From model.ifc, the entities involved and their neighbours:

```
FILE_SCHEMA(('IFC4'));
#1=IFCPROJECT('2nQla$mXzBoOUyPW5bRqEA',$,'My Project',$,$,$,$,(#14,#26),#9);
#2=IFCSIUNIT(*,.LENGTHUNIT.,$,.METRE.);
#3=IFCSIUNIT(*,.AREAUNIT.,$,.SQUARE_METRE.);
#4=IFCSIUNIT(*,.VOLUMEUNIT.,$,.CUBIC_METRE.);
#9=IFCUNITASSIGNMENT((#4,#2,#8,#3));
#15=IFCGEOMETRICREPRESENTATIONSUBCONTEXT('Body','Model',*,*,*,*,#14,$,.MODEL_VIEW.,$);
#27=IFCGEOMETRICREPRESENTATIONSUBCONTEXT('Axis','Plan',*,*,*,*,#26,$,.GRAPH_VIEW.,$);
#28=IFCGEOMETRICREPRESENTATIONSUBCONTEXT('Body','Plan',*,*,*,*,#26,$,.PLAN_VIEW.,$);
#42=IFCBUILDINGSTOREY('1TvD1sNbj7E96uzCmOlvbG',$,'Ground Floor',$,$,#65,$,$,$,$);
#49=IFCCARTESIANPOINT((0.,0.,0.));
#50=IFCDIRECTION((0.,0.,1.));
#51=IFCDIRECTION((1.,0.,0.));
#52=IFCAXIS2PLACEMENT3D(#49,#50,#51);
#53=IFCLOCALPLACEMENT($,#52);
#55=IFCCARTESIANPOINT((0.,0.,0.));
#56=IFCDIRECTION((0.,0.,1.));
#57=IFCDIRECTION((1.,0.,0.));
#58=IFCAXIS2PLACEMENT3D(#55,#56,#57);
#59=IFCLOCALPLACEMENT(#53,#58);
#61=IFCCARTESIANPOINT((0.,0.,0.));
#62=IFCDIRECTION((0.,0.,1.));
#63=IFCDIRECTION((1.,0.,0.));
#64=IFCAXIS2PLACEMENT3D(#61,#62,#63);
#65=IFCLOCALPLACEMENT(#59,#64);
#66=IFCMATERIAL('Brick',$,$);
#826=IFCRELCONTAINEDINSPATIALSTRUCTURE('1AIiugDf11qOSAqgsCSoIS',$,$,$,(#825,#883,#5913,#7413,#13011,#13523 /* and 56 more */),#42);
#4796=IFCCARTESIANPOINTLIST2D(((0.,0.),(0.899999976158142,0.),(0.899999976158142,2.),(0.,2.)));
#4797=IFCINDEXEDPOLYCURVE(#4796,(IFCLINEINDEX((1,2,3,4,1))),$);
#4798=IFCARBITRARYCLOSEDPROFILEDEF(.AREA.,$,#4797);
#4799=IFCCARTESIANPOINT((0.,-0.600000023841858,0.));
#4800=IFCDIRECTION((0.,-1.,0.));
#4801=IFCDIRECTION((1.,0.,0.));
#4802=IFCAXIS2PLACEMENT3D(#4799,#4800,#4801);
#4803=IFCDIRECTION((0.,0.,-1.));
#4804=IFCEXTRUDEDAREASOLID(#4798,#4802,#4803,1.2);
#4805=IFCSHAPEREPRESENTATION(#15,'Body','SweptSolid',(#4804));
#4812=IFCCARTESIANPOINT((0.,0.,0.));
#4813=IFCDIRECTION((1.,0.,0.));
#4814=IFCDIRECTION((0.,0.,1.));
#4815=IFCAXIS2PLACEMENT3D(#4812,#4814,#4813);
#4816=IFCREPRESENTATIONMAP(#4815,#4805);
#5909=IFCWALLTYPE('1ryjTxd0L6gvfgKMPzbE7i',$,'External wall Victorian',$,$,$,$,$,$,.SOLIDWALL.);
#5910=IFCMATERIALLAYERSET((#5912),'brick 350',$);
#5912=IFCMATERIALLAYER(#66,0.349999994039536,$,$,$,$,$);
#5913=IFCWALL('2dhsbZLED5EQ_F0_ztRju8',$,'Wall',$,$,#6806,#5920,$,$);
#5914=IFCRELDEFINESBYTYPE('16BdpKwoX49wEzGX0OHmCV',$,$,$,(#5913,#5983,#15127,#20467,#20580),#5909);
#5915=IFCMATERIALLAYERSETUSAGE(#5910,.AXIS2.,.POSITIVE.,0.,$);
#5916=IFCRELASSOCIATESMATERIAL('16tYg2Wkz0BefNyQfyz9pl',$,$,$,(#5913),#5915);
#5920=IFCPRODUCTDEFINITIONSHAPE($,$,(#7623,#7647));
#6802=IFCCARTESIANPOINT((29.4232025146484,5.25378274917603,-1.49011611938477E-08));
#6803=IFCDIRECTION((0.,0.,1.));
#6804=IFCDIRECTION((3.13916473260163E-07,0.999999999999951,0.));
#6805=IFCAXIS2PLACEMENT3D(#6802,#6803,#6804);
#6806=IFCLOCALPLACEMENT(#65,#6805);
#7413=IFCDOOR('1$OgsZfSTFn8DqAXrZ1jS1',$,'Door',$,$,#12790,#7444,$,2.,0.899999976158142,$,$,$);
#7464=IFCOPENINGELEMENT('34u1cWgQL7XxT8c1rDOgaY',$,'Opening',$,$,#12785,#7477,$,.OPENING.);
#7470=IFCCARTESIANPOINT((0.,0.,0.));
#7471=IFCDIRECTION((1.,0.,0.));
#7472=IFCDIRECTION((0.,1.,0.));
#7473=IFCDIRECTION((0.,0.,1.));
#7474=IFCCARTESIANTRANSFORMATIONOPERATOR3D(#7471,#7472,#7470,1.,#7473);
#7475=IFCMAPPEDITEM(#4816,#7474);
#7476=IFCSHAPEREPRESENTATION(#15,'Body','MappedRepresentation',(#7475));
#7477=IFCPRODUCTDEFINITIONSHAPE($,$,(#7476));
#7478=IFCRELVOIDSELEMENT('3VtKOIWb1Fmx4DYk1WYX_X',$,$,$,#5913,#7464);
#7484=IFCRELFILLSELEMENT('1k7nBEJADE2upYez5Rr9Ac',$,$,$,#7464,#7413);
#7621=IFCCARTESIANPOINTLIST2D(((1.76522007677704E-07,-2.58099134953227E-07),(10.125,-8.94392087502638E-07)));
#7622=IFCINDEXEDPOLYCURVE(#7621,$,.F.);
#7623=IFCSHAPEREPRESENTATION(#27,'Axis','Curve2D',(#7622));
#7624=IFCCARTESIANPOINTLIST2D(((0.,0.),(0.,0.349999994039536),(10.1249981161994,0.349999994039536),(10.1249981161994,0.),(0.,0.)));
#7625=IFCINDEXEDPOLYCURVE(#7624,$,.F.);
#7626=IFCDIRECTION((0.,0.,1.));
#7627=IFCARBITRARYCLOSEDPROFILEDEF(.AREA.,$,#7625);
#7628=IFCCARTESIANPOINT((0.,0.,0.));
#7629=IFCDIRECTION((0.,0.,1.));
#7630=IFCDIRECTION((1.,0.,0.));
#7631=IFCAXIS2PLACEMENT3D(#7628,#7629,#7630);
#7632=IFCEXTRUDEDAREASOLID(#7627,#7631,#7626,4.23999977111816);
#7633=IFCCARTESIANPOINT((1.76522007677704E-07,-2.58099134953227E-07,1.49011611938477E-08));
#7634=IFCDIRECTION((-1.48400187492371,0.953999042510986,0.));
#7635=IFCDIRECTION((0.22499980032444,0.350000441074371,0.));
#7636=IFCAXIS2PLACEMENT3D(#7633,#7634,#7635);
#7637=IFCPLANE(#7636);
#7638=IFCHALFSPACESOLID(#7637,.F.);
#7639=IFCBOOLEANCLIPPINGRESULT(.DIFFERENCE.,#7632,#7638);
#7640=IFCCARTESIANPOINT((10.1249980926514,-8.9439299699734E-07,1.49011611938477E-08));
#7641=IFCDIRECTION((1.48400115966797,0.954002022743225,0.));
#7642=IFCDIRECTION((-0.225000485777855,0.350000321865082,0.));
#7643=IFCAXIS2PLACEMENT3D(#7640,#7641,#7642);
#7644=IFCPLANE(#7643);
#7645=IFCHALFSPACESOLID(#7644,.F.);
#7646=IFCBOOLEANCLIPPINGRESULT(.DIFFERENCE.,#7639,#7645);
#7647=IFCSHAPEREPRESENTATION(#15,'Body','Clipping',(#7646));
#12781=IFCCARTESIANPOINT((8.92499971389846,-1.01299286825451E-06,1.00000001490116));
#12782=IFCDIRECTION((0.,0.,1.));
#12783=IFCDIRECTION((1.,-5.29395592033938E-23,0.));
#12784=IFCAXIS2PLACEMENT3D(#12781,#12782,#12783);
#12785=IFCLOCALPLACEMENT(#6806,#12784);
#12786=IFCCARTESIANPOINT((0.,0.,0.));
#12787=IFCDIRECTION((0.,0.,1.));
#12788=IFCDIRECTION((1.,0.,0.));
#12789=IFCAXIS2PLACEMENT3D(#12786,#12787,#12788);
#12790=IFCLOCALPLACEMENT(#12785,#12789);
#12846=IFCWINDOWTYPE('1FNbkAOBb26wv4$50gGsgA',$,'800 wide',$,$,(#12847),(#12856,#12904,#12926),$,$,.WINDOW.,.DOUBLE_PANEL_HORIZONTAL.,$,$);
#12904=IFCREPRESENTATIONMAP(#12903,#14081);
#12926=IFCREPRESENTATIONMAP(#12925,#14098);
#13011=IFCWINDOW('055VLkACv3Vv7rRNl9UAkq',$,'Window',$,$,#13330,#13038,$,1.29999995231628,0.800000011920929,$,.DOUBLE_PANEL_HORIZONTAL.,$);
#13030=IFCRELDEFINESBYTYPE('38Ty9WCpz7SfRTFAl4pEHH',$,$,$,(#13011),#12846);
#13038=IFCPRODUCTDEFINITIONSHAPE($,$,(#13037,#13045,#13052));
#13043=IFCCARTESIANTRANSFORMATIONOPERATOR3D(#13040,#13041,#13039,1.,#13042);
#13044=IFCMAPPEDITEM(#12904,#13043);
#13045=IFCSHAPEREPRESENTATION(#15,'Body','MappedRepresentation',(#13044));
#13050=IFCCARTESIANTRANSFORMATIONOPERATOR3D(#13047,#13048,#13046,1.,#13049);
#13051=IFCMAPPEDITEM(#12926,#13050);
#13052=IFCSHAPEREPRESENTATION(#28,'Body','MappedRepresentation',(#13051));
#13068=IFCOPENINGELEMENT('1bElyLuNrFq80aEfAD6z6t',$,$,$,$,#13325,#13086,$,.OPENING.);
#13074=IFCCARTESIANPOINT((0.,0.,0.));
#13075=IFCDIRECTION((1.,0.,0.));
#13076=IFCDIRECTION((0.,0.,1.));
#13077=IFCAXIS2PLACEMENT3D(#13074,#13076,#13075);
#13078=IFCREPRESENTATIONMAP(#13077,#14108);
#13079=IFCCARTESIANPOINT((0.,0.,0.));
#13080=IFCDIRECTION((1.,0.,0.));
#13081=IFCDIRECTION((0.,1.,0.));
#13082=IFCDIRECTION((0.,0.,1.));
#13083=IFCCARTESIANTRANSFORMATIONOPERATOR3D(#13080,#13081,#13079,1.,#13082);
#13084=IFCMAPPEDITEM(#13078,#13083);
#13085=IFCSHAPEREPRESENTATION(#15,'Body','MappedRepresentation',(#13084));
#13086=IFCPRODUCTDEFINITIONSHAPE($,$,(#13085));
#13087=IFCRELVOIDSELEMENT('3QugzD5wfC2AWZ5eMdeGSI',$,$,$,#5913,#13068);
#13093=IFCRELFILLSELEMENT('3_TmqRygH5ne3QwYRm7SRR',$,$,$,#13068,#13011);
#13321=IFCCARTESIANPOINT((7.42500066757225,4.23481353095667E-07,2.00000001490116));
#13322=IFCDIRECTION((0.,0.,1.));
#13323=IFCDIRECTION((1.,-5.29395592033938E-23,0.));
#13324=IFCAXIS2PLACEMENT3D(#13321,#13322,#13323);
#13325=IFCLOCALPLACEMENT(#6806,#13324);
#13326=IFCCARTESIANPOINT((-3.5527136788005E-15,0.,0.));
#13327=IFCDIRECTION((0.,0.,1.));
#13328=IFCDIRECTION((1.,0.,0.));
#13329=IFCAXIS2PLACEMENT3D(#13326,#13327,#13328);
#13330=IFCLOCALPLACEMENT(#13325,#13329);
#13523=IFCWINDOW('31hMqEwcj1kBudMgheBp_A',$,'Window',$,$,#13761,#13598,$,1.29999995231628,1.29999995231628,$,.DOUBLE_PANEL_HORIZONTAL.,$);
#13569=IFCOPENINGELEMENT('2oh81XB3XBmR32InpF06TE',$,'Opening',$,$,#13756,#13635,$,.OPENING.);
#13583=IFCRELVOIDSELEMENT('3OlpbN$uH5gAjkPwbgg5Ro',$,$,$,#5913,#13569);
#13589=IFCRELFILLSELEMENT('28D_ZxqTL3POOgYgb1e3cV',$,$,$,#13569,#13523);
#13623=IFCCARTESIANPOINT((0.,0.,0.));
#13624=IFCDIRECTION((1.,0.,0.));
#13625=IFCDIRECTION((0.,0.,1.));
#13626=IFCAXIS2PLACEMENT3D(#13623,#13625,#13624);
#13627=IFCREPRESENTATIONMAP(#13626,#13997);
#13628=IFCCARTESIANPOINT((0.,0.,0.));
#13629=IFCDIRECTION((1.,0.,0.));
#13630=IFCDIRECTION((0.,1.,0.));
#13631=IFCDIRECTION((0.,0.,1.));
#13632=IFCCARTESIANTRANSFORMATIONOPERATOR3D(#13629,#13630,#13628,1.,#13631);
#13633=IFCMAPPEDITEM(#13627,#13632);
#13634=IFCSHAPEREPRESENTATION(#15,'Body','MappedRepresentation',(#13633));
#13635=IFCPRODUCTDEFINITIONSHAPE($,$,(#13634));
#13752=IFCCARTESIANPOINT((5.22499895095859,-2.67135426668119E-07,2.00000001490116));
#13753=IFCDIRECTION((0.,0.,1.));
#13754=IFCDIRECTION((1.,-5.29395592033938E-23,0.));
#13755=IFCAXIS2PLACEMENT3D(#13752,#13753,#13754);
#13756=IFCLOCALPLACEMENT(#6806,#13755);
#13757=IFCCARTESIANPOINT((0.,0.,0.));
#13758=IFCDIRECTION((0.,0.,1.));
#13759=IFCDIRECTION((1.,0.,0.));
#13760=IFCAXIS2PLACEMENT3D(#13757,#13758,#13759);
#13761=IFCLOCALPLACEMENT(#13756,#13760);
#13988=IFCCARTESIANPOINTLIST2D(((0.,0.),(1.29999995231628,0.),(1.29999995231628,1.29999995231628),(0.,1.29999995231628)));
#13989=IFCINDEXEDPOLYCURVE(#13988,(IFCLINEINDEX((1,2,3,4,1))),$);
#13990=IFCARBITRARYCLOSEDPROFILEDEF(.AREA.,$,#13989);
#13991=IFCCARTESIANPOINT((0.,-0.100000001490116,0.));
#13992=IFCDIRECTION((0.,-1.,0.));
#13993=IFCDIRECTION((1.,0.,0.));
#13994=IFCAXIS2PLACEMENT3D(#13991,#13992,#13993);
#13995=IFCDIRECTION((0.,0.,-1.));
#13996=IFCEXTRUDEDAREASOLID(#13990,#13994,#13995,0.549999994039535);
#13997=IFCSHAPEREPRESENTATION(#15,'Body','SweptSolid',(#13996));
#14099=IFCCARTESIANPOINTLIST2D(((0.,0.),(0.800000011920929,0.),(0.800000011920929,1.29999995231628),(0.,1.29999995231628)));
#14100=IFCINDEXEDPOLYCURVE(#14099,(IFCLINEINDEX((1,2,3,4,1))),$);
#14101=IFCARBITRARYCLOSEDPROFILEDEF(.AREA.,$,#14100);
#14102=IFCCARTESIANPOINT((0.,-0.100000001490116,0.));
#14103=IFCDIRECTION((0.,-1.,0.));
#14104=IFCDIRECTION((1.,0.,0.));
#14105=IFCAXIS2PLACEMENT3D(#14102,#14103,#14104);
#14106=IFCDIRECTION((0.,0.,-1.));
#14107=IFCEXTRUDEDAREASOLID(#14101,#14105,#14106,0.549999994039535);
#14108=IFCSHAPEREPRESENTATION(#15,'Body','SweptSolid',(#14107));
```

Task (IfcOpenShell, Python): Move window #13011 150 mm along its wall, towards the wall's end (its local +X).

```python
import ifcopenshell
import ifcopenshell.api.geometry
import ifcopenshell.util.placement
import ifcopenshell.util.unit

model = ifcopenshell.open("model.ifc")
unit_scale = ifcopenshell.util.unit.calculate_unit_scale(model)

window = model.by_id(13011)
opening = window.FillsVoids[0].RelatingOpeningElement
wall = opening.VoidsElements[0].RelatingBuildingElement

wall_matrix = ifcopenshell.util.placement.get_local_placement(wall.ObjectPlacement)
shift = wall_matrix[:3, 0] * 0.15 / unit_scale
before = ifcopenshell.util.placement.get_local_placement(window.ObjectPlacement)[:3, 3].copy()

# The window is placed relative to its opening, so it follows when the opening moves.
matrix = ifcopenshell.util.placement.get_local_placement(opening.ObjectPlacement)
matrix[:3, 3] += shift
ifcopenshell.api.geometry.edit_object_placement(
    model, product=opening, matrix=matrix, is_si=False, should_transform_children=True
)

after = ifcopenshell.util.placement.get_local_placement(window.ObjectPlacement)[:3, 3]
print("window moved by", (after - before).round(3) + 0.0)

model.write("model-out.ifc")
```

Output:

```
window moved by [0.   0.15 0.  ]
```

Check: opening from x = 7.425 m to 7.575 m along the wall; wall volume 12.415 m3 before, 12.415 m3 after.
